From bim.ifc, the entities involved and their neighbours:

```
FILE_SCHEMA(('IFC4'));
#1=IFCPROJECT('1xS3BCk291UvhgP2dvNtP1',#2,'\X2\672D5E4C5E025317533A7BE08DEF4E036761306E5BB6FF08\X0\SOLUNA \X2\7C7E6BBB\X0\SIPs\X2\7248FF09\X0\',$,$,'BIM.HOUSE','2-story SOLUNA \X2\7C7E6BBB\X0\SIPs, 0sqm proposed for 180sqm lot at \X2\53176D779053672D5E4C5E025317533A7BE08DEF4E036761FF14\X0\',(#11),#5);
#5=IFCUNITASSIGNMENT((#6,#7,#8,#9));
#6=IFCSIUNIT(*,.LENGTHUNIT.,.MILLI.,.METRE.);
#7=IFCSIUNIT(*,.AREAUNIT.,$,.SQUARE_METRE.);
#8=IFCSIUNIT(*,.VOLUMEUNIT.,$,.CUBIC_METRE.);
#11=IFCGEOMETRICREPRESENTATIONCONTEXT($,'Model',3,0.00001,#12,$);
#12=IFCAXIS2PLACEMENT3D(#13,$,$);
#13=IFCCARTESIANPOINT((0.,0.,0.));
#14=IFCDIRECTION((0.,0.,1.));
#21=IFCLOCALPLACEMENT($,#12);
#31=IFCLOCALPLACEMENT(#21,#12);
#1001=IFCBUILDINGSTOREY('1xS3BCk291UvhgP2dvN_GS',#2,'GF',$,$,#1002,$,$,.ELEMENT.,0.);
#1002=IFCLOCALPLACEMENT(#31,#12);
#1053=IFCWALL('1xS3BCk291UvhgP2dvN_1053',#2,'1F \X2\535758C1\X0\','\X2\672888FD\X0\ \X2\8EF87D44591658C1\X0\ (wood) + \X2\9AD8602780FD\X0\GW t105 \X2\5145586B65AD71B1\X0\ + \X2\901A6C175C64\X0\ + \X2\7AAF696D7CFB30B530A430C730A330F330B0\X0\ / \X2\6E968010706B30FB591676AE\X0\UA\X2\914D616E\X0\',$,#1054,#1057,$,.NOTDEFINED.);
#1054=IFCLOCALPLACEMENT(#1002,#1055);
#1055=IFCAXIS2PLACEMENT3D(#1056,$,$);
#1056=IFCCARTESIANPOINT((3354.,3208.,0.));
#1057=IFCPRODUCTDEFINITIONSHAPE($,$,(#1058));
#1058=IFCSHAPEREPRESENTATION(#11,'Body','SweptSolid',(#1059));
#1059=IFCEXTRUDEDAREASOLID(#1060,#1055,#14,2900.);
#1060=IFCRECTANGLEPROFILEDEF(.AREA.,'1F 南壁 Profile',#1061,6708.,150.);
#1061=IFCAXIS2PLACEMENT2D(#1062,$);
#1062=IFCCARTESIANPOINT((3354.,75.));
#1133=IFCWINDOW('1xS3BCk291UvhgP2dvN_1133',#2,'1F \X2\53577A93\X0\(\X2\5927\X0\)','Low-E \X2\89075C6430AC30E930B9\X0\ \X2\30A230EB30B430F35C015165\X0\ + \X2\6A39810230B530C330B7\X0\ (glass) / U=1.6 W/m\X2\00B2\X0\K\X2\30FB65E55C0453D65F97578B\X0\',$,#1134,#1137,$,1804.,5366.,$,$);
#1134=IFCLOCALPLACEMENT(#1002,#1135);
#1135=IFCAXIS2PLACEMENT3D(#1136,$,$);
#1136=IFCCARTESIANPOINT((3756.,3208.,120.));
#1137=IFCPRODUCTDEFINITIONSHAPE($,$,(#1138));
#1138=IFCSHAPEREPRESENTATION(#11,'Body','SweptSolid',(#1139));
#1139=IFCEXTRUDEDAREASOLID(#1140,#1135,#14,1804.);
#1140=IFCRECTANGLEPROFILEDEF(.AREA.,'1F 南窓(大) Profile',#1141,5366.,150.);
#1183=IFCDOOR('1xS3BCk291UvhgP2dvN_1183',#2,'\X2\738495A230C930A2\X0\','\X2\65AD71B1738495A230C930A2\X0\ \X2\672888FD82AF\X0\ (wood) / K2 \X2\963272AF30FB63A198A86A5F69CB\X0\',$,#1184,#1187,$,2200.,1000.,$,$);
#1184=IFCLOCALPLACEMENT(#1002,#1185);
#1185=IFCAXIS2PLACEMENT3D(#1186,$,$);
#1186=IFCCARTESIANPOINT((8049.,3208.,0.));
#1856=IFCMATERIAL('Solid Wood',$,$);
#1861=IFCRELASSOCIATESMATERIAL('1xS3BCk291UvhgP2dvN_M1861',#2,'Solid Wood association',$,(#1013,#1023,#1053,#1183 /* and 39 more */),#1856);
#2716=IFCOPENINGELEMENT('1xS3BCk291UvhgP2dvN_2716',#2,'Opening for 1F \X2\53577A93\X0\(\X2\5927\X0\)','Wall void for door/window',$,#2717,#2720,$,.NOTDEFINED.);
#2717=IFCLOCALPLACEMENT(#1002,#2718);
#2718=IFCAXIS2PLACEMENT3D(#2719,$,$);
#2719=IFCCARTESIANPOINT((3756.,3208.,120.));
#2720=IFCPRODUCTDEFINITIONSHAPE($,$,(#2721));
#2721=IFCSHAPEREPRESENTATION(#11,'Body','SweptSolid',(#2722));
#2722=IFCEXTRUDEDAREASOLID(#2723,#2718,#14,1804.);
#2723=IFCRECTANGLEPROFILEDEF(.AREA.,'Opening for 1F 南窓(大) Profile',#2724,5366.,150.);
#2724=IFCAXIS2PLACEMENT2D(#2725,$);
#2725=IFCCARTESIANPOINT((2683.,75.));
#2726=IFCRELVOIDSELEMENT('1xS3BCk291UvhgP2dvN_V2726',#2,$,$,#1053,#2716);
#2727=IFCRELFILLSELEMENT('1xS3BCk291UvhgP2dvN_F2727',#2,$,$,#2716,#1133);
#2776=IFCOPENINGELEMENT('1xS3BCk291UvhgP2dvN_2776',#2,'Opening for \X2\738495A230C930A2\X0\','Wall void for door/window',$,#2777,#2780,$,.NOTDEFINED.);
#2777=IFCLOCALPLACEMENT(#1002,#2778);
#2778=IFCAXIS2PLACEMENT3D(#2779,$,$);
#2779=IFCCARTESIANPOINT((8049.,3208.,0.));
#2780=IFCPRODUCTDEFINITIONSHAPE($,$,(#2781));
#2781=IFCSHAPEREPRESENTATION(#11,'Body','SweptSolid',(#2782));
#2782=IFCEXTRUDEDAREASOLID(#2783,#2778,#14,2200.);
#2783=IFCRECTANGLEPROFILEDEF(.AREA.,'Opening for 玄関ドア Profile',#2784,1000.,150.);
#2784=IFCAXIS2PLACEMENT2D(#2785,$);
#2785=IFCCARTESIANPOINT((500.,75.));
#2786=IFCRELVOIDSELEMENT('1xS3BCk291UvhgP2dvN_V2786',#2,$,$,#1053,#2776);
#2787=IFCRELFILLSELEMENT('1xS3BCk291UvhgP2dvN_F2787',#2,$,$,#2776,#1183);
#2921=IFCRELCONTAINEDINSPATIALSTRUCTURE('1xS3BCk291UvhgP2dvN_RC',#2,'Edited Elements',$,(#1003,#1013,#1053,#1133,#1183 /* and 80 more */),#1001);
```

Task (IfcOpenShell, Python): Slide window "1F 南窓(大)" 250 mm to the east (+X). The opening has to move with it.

```python
import ifcopenshell
import ifcopenshell.api.geometry
import ifcopenshell.util.placement

model = ifcopenshell.open("bim.ifc")

window = model.by_guid("1xS3BCk291UvhgP2dvN_1133")
opening = window.FillsVoids[0].RelatingOpeningElement
wall = opening.VoidsElements[0].RelatingBuildingElement

wall_matrix = ifcopenshell.util.placement.get_local_placement(wall.ObjectPlacement)
shift = wall_matrix[:3, 0] * 250.0
before = ifcopenshell.util.placement.get_local_placement(window.ObjectPlacement)[:3, 3].copy()

# The window is not placed relative to its opening, so move both.
for product in (opening, window):
    matrix = ifcopenshell.util.placement.get_local_placement(product.ObjectPlacement)
    matrix[:3, 3] += shift
    ifcopenshell.api.geometry.edit_object_placement(model, product=product, matrix=matrix, is_si=False)

after = ifcopenshell.util.placement.get_local_placement(window.ObjectPlacement)[:3, 3]
print("window moved by", (after - before).round(3) + 0.0)

model.write("bim-out.ifc")
```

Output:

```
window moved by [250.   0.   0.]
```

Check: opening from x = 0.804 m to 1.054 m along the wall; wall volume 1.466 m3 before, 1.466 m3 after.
